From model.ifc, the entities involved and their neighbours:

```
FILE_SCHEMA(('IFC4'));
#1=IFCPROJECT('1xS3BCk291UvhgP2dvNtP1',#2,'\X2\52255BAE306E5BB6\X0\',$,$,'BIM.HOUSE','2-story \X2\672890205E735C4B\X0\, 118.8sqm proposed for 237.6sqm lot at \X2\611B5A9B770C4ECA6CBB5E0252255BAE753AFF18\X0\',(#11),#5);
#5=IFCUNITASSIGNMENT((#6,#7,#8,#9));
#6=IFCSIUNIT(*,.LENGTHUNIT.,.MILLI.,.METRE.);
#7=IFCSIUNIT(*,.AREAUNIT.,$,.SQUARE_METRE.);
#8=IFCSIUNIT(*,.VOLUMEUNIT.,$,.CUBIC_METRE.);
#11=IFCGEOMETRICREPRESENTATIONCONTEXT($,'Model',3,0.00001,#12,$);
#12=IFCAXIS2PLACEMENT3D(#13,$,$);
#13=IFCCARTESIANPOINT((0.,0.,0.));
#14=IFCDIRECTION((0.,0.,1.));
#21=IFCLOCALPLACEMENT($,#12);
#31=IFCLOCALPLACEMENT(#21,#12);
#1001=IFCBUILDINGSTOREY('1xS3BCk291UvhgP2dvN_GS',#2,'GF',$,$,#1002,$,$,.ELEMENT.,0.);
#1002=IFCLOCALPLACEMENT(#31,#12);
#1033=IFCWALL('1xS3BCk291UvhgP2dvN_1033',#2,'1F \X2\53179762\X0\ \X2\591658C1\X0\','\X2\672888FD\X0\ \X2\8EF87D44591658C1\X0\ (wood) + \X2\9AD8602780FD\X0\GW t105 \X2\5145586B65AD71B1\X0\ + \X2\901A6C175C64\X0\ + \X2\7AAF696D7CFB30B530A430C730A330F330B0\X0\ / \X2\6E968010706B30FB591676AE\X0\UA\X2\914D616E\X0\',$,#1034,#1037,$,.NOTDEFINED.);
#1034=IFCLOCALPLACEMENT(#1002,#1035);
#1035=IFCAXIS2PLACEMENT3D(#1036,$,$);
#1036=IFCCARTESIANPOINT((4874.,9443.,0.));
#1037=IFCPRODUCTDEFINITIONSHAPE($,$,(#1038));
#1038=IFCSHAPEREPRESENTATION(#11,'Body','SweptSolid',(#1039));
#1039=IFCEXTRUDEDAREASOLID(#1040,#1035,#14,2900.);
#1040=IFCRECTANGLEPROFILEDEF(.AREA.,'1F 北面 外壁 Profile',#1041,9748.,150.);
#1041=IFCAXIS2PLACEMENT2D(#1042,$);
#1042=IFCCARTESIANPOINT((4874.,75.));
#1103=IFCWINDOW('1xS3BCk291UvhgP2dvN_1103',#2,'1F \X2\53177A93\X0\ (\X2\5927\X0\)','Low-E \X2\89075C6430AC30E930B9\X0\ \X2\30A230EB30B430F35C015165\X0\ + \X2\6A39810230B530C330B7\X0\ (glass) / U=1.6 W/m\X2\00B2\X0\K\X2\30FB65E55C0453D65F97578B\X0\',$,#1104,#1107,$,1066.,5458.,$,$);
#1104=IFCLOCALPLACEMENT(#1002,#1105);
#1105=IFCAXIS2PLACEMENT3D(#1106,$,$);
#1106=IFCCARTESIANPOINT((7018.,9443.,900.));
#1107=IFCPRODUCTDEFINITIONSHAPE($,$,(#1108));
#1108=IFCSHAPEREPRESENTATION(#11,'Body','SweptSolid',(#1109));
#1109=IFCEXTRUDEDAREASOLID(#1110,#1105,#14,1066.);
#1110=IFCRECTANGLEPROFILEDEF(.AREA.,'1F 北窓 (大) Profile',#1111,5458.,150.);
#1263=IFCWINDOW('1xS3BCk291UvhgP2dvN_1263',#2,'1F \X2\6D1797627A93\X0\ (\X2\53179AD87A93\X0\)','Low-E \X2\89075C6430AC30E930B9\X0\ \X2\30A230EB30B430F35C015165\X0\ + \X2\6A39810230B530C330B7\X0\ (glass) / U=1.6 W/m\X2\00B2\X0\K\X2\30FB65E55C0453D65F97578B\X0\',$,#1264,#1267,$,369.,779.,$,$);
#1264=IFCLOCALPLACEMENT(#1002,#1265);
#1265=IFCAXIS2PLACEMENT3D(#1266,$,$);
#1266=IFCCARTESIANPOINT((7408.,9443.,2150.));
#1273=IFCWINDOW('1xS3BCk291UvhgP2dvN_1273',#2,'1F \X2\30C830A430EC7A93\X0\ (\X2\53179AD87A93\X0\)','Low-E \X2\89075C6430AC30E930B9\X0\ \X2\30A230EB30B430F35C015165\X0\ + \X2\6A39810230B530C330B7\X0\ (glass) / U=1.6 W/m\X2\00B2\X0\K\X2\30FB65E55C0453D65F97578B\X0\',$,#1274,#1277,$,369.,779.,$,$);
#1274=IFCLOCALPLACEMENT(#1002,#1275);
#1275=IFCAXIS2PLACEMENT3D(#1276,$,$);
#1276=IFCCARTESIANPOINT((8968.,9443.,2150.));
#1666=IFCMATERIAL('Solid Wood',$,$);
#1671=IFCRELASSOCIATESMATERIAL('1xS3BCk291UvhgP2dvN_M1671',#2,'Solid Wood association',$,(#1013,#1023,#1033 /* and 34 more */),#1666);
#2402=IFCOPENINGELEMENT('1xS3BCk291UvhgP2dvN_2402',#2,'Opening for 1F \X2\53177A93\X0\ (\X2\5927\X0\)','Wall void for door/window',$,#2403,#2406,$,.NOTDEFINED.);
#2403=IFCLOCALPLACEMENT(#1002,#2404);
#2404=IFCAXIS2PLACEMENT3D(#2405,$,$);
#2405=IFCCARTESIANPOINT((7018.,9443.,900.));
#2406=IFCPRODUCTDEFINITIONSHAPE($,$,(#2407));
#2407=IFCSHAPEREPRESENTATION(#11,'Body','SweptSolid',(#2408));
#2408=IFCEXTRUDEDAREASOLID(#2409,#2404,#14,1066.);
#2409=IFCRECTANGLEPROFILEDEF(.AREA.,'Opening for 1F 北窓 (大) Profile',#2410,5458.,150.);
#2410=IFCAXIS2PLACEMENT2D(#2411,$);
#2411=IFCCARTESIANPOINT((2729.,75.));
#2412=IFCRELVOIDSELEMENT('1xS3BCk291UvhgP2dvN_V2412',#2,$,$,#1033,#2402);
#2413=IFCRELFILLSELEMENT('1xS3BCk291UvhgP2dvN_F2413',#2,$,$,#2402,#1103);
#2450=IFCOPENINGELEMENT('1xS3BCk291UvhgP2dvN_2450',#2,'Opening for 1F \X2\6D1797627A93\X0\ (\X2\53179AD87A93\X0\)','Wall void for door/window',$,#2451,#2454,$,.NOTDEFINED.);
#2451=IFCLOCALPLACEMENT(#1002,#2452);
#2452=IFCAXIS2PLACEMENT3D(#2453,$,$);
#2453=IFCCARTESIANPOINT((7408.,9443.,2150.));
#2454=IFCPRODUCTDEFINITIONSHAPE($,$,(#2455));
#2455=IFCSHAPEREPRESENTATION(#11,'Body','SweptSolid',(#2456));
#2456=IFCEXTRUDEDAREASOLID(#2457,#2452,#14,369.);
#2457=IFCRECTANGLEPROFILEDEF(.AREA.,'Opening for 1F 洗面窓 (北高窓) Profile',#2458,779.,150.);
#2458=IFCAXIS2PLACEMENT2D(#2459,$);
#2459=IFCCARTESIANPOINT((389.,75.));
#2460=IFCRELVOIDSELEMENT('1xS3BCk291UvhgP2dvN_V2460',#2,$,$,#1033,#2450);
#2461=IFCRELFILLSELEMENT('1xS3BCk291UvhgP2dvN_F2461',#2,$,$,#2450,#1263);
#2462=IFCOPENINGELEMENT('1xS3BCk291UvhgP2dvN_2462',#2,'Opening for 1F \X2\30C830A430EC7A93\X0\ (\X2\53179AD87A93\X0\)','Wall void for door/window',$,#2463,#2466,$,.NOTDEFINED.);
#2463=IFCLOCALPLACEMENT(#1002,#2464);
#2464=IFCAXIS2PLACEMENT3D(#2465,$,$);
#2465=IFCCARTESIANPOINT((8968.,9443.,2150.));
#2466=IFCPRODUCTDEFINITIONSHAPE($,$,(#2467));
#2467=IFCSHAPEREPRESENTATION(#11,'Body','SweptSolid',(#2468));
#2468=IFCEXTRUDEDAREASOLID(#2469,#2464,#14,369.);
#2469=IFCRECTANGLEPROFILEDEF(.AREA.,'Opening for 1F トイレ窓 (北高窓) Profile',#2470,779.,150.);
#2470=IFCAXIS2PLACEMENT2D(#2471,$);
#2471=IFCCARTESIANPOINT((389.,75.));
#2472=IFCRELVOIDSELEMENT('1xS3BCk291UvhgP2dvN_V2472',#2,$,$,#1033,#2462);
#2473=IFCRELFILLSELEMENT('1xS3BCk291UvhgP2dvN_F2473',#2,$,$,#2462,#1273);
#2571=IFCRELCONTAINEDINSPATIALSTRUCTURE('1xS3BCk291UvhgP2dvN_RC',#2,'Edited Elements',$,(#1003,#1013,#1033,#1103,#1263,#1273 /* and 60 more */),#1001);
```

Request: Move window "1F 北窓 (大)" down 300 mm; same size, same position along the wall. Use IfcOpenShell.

```python
import numpy as np
import ifcopenshell
import ifcopenshell.api.geometry
import ifcopenshell.util.placement
import ifcopenshell.util.unit

model = ifcopenshell.open("model.ifc")
unit_scale = ifcopenshell.util.unit.calculate_unit_scale(model)

window = model.by_guid("1xS3BCk291UvhgP2dvN_1103")
opening = window.FillsVoids[0].RelatingOpeningElement
dz = -300.0

shift = np.array([0.0, 0.0, dz])
# The window is not placed relative to its opening, so move both.
for product in (opening, window):
    matrix = ifcopenshell.util.placement.get_local_placement(product.ObjectPlacement)
    matrix[:3, 3] += shift
    ifcopenshell.api.geometry.edit_object_placement(model, product=product, matrix=matrix, is_si=False)

print(f"moved by {dz * unit_scale:+.3f} m")

model.write("model-out.ifc")
```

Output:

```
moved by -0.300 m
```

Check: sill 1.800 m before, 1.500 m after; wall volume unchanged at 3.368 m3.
